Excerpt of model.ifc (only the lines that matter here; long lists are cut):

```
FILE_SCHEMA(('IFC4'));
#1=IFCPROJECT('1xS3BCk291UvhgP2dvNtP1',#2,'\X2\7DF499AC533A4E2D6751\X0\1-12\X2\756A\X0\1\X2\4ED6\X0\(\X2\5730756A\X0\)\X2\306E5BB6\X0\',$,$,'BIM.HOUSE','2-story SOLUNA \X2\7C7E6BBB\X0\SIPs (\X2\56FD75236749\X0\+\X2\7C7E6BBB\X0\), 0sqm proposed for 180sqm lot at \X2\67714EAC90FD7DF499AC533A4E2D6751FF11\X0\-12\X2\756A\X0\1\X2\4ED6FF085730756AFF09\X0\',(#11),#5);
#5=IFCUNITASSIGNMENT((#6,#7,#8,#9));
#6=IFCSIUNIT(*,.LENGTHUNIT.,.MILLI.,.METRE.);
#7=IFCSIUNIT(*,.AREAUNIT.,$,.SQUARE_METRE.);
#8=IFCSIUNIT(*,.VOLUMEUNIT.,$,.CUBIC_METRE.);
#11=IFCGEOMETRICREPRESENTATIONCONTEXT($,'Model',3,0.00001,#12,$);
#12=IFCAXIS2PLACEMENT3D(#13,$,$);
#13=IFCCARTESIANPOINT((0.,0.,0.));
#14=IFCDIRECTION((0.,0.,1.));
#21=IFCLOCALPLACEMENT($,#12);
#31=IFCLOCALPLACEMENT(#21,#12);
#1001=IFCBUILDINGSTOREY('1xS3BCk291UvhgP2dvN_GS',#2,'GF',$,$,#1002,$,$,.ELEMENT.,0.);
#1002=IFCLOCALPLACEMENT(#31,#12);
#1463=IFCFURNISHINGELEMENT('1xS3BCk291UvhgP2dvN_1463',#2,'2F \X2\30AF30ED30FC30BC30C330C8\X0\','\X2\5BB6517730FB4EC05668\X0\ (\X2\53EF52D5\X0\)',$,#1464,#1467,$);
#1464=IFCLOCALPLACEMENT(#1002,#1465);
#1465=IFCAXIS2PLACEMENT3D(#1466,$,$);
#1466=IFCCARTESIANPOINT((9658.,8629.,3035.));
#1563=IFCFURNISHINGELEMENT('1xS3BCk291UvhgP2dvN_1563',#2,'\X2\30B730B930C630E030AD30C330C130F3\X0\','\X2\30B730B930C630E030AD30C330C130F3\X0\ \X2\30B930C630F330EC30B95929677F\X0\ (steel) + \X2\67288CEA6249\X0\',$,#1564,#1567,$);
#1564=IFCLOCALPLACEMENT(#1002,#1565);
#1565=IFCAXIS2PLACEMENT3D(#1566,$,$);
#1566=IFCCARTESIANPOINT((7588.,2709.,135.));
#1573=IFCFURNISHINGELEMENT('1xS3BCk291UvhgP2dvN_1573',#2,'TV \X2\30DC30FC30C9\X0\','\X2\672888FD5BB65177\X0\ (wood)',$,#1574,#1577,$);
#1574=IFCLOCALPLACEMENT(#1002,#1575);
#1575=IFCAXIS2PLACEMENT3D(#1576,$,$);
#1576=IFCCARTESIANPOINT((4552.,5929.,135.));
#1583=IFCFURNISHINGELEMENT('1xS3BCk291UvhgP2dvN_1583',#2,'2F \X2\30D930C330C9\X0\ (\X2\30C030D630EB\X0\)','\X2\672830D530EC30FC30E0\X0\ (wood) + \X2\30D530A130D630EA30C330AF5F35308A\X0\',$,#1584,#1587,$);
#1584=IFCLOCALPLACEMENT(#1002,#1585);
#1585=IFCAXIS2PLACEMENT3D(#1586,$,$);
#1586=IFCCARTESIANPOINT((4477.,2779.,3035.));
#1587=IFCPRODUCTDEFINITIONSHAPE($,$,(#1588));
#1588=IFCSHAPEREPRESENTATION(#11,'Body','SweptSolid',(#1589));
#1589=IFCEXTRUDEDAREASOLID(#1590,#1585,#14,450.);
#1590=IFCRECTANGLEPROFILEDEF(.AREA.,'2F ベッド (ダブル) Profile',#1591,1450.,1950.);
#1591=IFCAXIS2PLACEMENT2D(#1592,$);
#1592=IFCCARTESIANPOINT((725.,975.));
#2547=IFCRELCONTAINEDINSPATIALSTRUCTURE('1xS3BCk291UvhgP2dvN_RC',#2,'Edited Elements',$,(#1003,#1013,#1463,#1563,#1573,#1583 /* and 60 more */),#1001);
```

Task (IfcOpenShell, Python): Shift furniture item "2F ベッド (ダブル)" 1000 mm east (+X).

```python
import ifcopenshell
import ifcopenshell.api.geometry
import ifcopenshell.util.placement
import ifcopenshell.util.unit

model = ifcopenshell.open("model.ifc")
unit_scale = ifcopenshell.util.unit.calculate_unit_scale(model)

item = model.by_guid("1xS3BCk291UvhgP2dvN_1583")
matrix = ifcopenshell.util.placement.get_local_placement(item.ObjectPlacement)
matrix[0, 3] += 1 / unit_scale
ifcopenshell.api.geometry.edit_object_placement(model, product=item, matrix=matrix, is_si=False)

print(ifcopenshell.util.placement.get_local_placement(item.ObjectPlacement).round(3) + 0.0)

model.write("model_rev.ifc")
```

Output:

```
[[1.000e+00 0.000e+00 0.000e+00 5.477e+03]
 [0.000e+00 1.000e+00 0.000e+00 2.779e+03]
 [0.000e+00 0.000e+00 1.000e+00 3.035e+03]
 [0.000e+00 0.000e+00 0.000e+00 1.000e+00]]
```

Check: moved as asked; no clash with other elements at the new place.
